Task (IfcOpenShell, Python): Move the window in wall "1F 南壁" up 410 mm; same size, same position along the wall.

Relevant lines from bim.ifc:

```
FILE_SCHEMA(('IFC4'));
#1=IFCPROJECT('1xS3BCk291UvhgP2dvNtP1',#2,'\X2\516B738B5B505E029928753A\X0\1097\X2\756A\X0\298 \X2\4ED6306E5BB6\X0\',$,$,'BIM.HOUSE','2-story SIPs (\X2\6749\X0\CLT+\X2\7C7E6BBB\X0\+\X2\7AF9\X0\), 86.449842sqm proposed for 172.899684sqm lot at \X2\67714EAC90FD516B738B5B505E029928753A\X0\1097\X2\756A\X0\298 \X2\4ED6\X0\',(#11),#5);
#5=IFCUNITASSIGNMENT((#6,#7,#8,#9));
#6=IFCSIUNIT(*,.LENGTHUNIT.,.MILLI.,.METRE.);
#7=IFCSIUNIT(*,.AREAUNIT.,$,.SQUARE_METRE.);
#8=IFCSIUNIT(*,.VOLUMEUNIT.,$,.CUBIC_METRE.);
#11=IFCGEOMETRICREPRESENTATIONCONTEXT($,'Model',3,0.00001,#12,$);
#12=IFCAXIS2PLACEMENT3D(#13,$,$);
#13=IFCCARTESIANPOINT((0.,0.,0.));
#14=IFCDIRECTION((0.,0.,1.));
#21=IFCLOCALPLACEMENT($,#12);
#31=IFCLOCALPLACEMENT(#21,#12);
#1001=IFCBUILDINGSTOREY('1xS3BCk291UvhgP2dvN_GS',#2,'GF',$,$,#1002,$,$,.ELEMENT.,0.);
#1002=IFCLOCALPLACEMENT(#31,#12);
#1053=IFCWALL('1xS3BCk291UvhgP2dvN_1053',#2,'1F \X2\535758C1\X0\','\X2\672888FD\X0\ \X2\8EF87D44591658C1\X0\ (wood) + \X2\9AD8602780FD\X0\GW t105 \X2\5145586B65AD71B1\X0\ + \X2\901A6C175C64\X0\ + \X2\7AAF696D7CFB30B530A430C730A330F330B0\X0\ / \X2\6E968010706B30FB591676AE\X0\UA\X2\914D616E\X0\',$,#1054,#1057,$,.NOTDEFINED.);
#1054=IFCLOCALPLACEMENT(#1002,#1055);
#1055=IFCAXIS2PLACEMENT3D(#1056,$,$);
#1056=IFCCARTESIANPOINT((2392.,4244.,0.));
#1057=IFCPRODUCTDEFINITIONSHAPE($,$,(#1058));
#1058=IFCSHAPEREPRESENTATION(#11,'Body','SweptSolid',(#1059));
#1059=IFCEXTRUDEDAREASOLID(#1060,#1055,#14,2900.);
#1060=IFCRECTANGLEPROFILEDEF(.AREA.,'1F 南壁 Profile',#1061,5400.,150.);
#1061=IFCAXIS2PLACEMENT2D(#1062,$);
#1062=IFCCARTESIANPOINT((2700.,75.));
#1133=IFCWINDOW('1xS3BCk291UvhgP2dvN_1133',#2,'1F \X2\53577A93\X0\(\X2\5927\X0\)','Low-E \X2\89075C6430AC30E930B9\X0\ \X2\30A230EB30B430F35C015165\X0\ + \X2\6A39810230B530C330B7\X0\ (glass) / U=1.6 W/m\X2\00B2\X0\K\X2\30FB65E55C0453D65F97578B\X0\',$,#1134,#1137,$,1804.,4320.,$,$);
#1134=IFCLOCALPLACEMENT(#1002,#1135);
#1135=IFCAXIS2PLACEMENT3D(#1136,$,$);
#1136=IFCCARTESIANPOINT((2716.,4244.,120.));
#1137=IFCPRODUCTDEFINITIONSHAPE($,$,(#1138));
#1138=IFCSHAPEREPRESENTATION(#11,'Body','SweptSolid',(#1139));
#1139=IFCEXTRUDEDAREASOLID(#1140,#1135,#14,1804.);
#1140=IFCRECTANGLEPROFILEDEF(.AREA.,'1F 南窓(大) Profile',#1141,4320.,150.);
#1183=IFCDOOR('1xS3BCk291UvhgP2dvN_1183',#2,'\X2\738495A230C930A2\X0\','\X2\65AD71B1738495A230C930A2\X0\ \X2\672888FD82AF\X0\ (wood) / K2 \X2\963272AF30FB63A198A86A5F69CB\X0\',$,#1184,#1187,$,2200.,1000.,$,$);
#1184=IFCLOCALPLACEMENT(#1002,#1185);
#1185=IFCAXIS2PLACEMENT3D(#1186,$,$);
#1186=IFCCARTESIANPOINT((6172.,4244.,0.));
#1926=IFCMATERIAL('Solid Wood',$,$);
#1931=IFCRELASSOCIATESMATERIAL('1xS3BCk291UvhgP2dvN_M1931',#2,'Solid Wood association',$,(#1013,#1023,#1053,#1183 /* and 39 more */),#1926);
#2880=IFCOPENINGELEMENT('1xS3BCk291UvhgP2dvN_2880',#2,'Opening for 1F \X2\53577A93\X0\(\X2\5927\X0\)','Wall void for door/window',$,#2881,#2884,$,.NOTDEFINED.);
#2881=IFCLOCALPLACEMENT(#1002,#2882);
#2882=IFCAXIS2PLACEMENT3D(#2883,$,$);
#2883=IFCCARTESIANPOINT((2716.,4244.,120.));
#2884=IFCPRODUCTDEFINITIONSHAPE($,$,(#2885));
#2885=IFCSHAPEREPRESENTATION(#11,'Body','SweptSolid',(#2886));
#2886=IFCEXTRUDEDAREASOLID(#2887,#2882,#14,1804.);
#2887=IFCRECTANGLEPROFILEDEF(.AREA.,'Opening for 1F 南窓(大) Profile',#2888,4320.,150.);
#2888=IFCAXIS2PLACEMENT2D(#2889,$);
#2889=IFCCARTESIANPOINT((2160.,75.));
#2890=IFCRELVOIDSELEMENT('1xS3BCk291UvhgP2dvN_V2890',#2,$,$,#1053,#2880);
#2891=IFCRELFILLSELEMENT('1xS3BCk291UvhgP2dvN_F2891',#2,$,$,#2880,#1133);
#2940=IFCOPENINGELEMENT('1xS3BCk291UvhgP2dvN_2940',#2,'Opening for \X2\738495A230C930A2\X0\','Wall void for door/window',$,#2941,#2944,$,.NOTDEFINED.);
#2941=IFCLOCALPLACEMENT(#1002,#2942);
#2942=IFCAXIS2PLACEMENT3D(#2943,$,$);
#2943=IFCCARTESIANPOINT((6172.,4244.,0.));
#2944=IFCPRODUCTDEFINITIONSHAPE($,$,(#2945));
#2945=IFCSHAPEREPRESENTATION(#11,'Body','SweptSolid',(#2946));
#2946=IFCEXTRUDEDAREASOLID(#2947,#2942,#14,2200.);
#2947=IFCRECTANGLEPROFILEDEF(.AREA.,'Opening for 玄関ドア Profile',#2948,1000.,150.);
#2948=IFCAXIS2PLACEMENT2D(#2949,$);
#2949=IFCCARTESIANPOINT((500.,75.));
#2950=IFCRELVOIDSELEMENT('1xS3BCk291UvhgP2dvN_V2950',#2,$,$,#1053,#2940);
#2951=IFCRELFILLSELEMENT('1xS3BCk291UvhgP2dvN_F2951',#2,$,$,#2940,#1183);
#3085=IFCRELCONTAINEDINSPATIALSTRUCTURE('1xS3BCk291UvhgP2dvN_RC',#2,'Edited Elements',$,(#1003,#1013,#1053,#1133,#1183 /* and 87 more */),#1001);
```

```python
import numpy as np
import ifcopenshell
import ifcopenshell.api.geometry
import ifcopenshell.util.placement
import ifcopenshell.util.unit

model = ifcopenshell.open("bim.ifc")
unit_scale = ifcopenshell.util.unit.calculate_unit_scale(model)

window = model.by_guid("1xS3BCk291UvhgP2dvN_1133")
opening = window.FillsVoids[0].RelatingOpeningElement
dz = 0.41 / unit_scale

shift = np.array([0.0, 0.0, dz])
# The window is not placed relative to its opening, so move both.
for product in (opening, window):
    matrix = ifcopenshell.util.placement.get_local_placement(product.ObjectPlacement)
    matrix[:3, 3] += shift
    ifcopenshell.api.geometry.edit_object_placement(model, product=product, matrix=matrix, is_si=False)

print(f"moved by {dz * unit_scale:+.3f} m")

model.write("bim_updated.ifc")
```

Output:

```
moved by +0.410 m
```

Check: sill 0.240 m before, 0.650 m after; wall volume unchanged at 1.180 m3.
